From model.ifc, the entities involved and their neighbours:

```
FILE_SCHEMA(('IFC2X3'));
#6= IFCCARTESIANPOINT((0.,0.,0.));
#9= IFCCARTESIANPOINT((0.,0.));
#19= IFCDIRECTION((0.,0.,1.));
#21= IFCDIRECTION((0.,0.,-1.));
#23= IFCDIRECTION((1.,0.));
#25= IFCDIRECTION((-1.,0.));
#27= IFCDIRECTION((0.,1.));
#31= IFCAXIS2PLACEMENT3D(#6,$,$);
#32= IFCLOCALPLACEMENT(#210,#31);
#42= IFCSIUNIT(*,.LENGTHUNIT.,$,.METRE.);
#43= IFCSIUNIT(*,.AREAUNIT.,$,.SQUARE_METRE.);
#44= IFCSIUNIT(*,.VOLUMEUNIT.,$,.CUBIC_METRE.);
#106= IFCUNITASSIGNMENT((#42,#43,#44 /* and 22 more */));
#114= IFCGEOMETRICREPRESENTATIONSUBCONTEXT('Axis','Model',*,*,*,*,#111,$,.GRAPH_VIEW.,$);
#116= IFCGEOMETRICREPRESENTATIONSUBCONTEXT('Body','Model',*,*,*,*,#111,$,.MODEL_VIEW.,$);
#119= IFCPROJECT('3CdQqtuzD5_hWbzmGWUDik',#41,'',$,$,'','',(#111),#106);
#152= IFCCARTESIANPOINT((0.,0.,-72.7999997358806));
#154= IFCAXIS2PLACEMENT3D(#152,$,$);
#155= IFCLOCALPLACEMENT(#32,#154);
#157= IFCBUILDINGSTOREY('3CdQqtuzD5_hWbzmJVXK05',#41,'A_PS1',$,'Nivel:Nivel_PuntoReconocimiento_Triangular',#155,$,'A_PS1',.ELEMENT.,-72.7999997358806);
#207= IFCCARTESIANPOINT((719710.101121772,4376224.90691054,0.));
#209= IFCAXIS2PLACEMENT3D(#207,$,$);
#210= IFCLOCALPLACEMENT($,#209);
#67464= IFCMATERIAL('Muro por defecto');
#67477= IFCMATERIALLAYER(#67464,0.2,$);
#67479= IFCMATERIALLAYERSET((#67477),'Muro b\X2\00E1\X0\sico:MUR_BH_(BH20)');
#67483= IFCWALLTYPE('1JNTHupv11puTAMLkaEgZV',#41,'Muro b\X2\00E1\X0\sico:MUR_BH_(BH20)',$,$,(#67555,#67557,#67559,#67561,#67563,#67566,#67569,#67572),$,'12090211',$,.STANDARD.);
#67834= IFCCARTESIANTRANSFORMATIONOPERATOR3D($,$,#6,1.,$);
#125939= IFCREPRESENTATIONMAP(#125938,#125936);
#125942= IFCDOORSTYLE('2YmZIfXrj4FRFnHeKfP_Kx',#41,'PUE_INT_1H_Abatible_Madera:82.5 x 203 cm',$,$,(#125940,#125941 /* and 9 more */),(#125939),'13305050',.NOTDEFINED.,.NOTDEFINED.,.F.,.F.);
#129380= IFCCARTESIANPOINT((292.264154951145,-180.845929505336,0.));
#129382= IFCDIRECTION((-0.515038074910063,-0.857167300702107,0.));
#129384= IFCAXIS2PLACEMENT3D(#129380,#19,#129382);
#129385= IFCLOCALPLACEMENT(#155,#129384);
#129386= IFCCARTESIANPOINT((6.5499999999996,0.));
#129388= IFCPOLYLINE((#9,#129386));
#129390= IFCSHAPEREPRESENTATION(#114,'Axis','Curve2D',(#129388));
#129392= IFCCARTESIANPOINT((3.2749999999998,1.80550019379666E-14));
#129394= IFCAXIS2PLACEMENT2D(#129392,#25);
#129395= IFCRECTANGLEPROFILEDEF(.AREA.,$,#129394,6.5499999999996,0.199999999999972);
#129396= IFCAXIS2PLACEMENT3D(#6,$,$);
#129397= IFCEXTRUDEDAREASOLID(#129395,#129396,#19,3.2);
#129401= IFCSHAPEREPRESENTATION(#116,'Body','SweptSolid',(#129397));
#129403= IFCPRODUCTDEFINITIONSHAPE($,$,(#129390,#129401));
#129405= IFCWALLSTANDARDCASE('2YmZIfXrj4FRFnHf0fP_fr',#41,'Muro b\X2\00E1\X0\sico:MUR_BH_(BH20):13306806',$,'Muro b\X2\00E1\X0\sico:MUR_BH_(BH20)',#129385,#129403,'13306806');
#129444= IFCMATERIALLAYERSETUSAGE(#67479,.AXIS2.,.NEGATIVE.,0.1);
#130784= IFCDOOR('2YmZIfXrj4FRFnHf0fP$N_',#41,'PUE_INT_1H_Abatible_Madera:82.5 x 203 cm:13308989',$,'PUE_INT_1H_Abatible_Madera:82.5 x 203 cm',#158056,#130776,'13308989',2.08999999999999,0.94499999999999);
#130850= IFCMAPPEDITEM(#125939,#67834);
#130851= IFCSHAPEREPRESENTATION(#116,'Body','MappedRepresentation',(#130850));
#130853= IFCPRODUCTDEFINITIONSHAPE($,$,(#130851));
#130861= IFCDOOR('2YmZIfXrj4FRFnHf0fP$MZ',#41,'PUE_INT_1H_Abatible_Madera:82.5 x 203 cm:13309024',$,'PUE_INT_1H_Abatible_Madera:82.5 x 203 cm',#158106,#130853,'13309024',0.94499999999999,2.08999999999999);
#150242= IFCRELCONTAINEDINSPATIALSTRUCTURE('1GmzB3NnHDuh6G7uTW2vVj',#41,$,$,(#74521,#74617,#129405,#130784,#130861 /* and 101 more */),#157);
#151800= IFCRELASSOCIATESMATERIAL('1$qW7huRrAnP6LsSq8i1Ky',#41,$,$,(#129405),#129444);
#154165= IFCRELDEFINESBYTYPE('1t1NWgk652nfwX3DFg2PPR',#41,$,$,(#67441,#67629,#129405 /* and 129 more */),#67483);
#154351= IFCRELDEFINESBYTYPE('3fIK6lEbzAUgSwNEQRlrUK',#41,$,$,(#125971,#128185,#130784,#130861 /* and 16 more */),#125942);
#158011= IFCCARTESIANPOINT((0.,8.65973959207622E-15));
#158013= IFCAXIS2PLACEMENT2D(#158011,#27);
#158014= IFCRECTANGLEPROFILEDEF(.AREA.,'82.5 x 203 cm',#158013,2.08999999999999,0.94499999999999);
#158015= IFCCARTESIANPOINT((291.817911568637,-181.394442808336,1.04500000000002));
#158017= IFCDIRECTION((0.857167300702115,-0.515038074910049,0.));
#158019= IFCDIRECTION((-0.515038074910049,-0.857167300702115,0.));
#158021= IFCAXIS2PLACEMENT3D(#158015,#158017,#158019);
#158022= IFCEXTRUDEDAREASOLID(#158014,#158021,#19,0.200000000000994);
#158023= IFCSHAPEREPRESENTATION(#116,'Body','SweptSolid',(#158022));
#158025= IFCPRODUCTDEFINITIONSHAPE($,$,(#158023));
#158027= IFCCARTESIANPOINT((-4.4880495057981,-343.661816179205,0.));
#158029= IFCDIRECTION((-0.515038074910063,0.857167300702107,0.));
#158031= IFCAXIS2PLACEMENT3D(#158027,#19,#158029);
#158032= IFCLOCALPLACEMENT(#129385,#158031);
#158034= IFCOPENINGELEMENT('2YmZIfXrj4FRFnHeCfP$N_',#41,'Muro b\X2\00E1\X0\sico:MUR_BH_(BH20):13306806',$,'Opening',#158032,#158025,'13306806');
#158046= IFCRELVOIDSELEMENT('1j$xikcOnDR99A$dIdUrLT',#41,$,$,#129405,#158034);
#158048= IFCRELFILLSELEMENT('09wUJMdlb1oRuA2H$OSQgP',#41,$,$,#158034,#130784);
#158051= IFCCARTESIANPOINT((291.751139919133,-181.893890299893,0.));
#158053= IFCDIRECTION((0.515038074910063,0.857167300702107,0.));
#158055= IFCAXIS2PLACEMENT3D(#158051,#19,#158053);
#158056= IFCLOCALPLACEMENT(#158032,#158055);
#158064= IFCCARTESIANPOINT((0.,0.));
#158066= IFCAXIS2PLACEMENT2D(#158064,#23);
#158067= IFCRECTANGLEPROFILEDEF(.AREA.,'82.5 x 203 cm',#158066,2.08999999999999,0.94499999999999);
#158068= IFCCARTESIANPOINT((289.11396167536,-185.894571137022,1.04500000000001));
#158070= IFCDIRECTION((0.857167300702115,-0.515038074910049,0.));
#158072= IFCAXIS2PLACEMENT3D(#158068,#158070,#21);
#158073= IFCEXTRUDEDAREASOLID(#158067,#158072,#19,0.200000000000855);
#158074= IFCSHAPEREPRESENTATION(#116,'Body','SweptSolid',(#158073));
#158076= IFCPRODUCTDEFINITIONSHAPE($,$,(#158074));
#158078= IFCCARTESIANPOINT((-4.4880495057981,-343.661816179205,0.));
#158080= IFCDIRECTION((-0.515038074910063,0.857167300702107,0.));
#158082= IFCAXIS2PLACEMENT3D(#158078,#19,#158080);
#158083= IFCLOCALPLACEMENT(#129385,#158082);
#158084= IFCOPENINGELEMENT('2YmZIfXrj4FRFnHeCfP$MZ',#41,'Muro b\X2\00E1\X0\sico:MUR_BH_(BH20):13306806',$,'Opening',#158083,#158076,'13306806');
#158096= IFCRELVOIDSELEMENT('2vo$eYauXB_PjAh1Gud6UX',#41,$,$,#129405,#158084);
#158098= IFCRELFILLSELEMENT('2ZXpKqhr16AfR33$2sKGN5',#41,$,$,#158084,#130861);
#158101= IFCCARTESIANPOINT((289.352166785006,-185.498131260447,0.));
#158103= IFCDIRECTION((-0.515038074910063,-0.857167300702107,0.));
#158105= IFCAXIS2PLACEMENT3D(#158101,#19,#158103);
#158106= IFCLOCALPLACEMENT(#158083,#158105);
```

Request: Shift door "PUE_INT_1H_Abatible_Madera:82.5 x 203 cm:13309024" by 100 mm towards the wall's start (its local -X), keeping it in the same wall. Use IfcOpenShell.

```python
import ifcopenshell
import ifcopenshell.api.geometry
import ifcopenshell.util.placement
import ifcopenshell.util.unit

model = ifcopenshell.open("model.ifc")
unit_scale = ifcopenshell.util.unit.calculate_unit_scale(model)

door = model.by_guid("2YmZIfXrj4FRFnHf0fP$MZ")
opening = door.FillsVoids[0].RelatingOpeningElement
wall = opening.VoidsElements[0].RelatingBuildingElement

wall_matrix = ifcopenshell.util.placement.get_local_placement(wall.ObjectPlacement)
shift = wall_matrix[:3, 0] * -0.1 / unit_scale
before = ifcopenshell.util.placement.get_local_placement(door.ObjectPlacement)[:3, 3].copy()

# The door is placed relative to its opening, so it follows when the opening moves.
matrix = ifcopenshell.util.placement.get_local_placement(opening.ObjectPlacement)
matrix[:3, 3] += shift
ifcopenshell.api.geometry.edit_object_placement(
    model, product=opening, matrix=matrix, is_si=False, should_transform_children=True
)

after = ifcopenshell.util.placement.get_local_placement(door.ObjectPlacement)[:3, 3]
print("door moved by", (after - before).round(3) + 0.0)

model.write("model_v2.ifc")
```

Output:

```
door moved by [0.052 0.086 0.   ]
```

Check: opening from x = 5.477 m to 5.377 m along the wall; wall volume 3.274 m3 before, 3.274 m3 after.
